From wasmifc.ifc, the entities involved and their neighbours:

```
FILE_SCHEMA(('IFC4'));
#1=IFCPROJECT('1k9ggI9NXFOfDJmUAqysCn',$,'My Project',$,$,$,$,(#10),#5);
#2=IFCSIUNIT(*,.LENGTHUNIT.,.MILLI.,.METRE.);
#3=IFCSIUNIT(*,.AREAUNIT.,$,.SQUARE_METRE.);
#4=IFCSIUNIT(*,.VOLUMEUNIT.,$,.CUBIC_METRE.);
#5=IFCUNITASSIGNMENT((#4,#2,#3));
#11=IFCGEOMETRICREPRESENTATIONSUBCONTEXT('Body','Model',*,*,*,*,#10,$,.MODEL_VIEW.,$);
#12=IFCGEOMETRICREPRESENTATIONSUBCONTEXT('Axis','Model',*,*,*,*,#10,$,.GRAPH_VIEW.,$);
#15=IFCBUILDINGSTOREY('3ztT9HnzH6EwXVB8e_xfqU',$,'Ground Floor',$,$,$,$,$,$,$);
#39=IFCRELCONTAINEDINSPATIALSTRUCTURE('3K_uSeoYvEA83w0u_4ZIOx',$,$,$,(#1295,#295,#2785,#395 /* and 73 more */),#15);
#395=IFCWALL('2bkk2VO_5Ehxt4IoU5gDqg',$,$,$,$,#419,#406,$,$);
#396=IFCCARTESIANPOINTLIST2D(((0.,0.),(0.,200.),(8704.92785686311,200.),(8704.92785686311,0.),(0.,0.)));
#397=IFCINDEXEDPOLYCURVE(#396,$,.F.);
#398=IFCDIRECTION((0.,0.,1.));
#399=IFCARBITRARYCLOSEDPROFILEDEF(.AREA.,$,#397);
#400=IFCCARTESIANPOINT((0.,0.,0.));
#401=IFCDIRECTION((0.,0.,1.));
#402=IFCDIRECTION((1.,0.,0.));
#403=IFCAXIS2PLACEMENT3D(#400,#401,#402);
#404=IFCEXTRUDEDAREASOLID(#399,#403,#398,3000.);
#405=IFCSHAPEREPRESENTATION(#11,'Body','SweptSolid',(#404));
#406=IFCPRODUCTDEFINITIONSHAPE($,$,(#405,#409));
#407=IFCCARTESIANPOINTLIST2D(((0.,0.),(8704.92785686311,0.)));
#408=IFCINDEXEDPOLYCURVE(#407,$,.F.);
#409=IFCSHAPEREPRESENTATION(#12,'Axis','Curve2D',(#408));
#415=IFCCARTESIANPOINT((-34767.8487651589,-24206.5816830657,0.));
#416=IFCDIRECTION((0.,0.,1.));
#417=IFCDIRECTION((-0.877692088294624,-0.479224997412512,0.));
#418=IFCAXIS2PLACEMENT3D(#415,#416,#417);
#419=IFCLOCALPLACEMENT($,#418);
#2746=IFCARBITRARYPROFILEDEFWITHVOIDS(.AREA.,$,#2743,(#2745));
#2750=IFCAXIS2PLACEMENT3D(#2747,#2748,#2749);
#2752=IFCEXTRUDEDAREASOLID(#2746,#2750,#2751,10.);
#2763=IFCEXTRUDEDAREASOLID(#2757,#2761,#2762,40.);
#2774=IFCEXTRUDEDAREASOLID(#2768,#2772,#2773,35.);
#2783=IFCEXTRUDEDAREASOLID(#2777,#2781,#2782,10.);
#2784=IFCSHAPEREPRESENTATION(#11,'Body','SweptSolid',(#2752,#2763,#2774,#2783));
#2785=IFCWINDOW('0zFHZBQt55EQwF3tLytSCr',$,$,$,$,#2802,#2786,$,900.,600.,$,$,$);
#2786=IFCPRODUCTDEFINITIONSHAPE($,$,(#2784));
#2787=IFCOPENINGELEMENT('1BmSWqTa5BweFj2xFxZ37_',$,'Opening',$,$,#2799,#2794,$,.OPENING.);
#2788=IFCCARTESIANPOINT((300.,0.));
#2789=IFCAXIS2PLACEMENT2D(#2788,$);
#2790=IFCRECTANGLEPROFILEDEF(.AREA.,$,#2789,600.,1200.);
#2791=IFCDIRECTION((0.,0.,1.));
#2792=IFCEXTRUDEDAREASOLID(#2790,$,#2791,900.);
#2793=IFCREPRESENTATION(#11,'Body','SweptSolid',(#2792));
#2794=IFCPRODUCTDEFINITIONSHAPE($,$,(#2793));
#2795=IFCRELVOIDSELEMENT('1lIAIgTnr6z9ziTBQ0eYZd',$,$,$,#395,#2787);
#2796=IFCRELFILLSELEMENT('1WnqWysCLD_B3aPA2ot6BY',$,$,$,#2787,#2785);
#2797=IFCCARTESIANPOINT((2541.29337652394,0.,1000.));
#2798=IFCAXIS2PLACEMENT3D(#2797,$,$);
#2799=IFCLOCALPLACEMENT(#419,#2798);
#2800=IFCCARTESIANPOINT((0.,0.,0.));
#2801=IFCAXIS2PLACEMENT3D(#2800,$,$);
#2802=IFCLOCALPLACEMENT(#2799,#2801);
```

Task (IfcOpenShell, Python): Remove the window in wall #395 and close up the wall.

```python
import ifcopenshell
import ifcopenshell.api.feature
import ifcopenshell.api.root
import ifcopenshell.geom
import ifcopenshell.util.shape

model = ifcopenshell.open("wasmifc.ifc")
settings = ifcopenshell.geom.settings()


def volume(element):
    """Net volume in cubic metres, openings subtracted."""
    shape = ifcopenshell.geom.create_shape(settings, element)
    return ifcopenshell.util.shape.get_volume(shape.geometry)


window = model.by_guid("0zFHZBQt55EQwF3tLytSCr")
opening = window.FillsVoids[0].RelatingOpeningElement
wall = opening.VoidsElements[0].RelatingBuildingElement
before = volume(wall)

ifcopenshell.api.root.remove_product(model, product=window)
ifcopenshell.api.feature.remove_feature(model, feature=opening)

after = volume(wall)

print(f"wall volume {before:.3f} -> {after:.3f} m3")

model.write("wasmifc-out.ifc")
```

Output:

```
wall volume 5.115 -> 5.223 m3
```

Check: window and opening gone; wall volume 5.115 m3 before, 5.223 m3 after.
